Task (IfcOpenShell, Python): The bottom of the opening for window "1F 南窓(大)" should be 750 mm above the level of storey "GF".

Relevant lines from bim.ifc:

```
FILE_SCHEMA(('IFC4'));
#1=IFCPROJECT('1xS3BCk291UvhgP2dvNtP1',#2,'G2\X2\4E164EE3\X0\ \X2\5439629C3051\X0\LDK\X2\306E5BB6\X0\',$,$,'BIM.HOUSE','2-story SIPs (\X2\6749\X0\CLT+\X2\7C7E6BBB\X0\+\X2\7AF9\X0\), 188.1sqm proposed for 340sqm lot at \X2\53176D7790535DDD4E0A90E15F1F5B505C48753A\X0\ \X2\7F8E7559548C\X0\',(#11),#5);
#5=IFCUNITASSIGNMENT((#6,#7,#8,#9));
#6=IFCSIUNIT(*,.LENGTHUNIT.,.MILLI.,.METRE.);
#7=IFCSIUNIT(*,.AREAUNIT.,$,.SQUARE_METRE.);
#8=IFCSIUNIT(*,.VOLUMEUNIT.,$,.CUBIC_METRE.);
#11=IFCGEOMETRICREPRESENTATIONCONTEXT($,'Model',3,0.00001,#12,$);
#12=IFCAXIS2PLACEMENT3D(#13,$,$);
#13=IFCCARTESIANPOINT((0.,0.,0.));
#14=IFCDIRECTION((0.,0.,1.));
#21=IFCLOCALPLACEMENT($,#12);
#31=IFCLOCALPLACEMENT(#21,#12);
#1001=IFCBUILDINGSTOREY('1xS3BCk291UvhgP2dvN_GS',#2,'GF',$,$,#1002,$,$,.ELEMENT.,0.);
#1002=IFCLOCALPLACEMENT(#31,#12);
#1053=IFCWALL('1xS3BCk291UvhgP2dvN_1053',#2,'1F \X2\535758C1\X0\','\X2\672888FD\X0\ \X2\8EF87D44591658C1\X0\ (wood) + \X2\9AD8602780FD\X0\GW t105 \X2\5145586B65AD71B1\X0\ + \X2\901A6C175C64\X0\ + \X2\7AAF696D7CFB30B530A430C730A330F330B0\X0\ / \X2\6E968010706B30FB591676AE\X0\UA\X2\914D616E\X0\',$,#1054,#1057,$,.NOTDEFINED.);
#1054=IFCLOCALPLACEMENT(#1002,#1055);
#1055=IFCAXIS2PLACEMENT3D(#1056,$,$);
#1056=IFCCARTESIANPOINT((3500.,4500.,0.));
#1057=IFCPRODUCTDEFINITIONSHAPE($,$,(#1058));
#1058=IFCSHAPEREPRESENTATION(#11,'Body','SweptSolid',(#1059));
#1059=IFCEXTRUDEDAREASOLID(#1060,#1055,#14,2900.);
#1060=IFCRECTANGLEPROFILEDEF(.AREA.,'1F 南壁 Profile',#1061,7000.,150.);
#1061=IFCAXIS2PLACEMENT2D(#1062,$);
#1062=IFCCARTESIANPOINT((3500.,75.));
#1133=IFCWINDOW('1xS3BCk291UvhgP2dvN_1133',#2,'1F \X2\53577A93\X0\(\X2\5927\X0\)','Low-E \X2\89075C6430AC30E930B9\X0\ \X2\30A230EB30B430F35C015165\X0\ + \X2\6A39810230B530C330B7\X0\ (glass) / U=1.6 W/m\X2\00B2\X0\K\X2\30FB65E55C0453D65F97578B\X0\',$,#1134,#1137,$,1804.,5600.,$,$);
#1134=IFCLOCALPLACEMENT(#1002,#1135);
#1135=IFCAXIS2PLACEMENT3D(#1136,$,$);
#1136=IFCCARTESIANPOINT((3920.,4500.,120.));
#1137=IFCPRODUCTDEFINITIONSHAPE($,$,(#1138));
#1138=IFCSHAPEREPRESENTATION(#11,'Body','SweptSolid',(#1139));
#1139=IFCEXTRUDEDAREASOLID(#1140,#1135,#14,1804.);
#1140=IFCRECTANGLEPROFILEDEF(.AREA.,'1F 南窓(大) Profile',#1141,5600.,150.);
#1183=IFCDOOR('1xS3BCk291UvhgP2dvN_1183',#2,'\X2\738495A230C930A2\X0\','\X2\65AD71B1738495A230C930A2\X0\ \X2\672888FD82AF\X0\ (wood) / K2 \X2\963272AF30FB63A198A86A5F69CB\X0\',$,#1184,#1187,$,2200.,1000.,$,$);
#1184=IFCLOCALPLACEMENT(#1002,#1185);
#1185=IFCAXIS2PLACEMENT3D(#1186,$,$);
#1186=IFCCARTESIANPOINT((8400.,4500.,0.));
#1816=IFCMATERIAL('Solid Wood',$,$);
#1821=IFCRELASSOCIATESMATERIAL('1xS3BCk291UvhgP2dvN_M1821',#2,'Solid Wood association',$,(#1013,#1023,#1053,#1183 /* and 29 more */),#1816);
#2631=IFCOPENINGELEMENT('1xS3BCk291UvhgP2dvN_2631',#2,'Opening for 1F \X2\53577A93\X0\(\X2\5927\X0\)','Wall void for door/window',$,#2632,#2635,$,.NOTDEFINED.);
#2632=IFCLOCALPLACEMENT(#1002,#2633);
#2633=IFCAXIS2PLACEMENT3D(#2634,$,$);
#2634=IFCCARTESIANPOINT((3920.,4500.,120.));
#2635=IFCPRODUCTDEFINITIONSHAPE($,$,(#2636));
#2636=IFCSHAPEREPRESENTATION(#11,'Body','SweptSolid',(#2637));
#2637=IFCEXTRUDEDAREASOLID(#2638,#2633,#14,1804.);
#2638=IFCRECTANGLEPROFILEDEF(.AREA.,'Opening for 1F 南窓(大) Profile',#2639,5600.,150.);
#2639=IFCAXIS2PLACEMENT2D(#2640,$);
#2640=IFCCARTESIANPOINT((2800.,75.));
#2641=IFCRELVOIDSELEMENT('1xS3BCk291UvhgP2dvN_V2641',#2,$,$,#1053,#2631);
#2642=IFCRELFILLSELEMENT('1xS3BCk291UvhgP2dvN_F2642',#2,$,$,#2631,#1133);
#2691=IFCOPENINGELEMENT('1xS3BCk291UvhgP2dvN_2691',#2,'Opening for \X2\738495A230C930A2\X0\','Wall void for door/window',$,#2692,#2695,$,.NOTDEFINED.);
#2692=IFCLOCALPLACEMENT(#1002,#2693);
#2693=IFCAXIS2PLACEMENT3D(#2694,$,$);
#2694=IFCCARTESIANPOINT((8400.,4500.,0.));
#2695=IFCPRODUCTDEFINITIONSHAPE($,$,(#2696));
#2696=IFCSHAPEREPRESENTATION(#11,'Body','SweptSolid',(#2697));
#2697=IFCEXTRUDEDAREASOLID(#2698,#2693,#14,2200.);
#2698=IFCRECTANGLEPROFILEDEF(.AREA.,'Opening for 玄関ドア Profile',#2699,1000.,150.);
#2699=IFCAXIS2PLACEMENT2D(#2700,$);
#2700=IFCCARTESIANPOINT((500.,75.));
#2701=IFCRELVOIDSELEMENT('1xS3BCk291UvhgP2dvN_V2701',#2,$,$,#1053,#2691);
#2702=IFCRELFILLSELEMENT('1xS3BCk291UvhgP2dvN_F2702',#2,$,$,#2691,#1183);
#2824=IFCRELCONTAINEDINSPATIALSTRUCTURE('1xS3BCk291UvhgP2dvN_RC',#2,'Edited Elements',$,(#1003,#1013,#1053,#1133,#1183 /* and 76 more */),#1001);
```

```python
import numpy as np
import ifcopenshell
import ifcopenshell.api.geometry
import ifcopenshell.geom
import ifcopenshell.util.element
import ifcopenshell.util.placement
import ifcopenshell.util.shape
import ifcopenshell.util.unit

model = ifcopenshell.open("bim.ifc")
unit_scale = ifcopenshell.util.unit.calculate_unit_scale(model)

window = model.by_guid("1xS3BCk291UvhgP2dvN_1133")
opening = window.FillsVoids[0].RelatingOpeningElement
storey = ifcopenshell.util.element.get_container(window, ifc_class="IfcBuildingStorey")
level = ifcopenshell.util.placement.get_local_placement(storey.ObjectPlacement)[2, 3]

# The opening's origin need not be at the sill, so measure its lowest point.
shape = ifcopenshell.geom.create_shape(ifcopenshell.geom.settings(), opening)
bottom = ifcopenshell.util.shape.get_shape_bottom_elevation(shape, shape.geometry) / unit_scale
dz = level + 750.0 - bottom

shift = np.array([0.0, 0.0, dz])
# The window is not placed relative to its opening, so move both.
for product in (opening, window):
    matrix = ifcopenshell.util.placement.get_local_placement(product.ObjectPlacement)
    matrix[:3, 3] += shift
    ifcopenshell.api.geometry.edit_object_placement(model, product=product, matrix=matrix, is_si=False)

print(f"moved by {dz * unit_scale:+.3f} m")

model.write("bim_edited.ifc")
```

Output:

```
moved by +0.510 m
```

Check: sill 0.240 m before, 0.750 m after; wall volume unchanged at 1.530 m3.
